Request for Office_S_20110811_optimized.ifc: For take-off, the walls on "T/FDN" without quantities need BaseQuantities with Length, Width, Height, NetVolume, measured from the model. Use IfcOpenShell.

First a look at what the model holds.

```python
import ifcopenshell
import ifcopenshell.util.element
import ifcopenshell.util.unit

model = ifcopenshell.open("Office_S_20110811_optimized.ifc")
print(model.schema)
for unit_type in ("LENGTHUNIT", "AREAUNIT", "VOLUMEUNIT"):
    print(unit_type, ifcopenshell.util.unit.calculate_unit_scale(model, unit_type))
storey = next(s for s in model.by_type("IfcBuildingStorey") if s.Name == "T/FDN")
walls = [e for e in ifcopenshell.util.element.get_decomposition(storey) if e.is_a("IfcWall")]
for e in sorted(walls, key=lambda e: e.id()):
    print(e.id(), e.is_a(), e.Name, list(ifcopenshell.util.element.get_psets(e, qtos_only=True)), sep=" | ")
```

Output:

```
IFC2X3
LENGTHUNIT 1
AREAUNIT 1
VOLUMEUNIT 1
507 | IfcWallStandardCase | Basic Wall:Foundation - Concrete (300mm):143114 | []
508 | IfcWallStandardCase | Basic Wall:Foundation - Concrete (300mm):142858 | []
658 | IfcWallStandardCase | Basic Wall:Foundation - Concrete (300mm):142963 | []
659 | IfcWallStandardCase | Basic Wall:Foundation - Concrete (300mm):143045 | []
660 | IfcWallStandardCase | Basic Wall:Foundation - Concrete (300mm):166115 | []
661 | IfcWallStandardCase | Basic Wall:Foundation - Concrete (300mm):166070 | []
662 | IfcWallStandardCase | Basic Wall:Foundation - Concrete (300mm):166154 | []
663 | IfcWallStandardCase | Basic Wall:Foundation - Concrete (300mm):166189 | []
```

```python
import ifcopenshell
import ifcopenshell.api.pset
import ifcopenshell.geom
import ifcopenshell.util.element
import ifcopenshell.util.shape
import ifcopenshell.util.unit

model = ifcopenshell.open("Office_S_20110811_optimized.ifc")
unit_scale = ifcopenshell.util.unit.calculate_unit_scale(model)
volume_scale = ifcopenshell.util.unit.calculate_unit_scale(model, "VOLUMEUNIT")
settings = ifcopenshell.geom.settings()

storey = next(s for s in model.by_type("IfcBuildingStorey") if s.Name == "T/FDN")
walls = [e for e in ifcopenshell.util.element.get_decomposition(storey) if e.is_a("IfcWall")]

for e in sorted(walls, key=lambda e: e.id()):
    if ifcopenshell.util.element.get_psets(e, qtos_only=True, should_inherit=False):
        continue
    # Geometry comes back in metres, in the element's own axes.
    shape = ifcopenshell.geom.create_shape(settings, e)
    values = {
        "Length": ifcopenshell.util.shape.get_x(shape.geometry) / unit_scale,
        "Width": ifcopenshell.util.shape.get_y(shape.geometry) / unit_scale,
        "Height": ifcopenshell.util.shape.get_z(shape.geometry) / unit_scale,
        "NetVolume": ifcopenshell.util.shape.get_volume(shape.geometry) / volume_scale,
    }
    qto = ifcopenshell.api.pset.add_qto(model, product=e, name="BaseQuantities")
    ifcopenshell.api.pset.edit_qto(model, qto=qto, properties=values)
    print(e.id(), {k: round(v, 3) for k, v in values.items()})

model.write("Office_S_20110811_optimized_v2.ifc")
```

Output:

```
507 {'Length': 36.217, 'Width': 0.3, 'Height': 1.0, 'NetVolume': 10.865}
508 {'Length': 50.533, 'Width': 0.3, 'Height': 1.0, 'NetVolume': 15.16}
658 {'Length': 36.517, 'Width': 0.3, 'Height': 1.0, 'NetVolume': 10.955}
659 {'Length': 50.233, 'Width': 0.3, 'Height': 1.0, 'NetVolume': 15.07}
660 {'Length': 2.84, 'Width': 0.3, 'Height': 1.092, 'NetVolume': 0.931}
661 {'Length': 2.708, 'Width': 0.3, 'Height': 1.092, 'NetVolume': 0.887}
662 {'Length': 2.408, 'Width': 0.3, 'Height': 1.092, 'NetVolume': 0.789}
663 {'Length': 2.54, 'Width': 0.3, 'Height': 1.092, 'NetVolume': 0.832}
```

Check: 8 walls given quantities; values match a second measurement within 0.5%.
